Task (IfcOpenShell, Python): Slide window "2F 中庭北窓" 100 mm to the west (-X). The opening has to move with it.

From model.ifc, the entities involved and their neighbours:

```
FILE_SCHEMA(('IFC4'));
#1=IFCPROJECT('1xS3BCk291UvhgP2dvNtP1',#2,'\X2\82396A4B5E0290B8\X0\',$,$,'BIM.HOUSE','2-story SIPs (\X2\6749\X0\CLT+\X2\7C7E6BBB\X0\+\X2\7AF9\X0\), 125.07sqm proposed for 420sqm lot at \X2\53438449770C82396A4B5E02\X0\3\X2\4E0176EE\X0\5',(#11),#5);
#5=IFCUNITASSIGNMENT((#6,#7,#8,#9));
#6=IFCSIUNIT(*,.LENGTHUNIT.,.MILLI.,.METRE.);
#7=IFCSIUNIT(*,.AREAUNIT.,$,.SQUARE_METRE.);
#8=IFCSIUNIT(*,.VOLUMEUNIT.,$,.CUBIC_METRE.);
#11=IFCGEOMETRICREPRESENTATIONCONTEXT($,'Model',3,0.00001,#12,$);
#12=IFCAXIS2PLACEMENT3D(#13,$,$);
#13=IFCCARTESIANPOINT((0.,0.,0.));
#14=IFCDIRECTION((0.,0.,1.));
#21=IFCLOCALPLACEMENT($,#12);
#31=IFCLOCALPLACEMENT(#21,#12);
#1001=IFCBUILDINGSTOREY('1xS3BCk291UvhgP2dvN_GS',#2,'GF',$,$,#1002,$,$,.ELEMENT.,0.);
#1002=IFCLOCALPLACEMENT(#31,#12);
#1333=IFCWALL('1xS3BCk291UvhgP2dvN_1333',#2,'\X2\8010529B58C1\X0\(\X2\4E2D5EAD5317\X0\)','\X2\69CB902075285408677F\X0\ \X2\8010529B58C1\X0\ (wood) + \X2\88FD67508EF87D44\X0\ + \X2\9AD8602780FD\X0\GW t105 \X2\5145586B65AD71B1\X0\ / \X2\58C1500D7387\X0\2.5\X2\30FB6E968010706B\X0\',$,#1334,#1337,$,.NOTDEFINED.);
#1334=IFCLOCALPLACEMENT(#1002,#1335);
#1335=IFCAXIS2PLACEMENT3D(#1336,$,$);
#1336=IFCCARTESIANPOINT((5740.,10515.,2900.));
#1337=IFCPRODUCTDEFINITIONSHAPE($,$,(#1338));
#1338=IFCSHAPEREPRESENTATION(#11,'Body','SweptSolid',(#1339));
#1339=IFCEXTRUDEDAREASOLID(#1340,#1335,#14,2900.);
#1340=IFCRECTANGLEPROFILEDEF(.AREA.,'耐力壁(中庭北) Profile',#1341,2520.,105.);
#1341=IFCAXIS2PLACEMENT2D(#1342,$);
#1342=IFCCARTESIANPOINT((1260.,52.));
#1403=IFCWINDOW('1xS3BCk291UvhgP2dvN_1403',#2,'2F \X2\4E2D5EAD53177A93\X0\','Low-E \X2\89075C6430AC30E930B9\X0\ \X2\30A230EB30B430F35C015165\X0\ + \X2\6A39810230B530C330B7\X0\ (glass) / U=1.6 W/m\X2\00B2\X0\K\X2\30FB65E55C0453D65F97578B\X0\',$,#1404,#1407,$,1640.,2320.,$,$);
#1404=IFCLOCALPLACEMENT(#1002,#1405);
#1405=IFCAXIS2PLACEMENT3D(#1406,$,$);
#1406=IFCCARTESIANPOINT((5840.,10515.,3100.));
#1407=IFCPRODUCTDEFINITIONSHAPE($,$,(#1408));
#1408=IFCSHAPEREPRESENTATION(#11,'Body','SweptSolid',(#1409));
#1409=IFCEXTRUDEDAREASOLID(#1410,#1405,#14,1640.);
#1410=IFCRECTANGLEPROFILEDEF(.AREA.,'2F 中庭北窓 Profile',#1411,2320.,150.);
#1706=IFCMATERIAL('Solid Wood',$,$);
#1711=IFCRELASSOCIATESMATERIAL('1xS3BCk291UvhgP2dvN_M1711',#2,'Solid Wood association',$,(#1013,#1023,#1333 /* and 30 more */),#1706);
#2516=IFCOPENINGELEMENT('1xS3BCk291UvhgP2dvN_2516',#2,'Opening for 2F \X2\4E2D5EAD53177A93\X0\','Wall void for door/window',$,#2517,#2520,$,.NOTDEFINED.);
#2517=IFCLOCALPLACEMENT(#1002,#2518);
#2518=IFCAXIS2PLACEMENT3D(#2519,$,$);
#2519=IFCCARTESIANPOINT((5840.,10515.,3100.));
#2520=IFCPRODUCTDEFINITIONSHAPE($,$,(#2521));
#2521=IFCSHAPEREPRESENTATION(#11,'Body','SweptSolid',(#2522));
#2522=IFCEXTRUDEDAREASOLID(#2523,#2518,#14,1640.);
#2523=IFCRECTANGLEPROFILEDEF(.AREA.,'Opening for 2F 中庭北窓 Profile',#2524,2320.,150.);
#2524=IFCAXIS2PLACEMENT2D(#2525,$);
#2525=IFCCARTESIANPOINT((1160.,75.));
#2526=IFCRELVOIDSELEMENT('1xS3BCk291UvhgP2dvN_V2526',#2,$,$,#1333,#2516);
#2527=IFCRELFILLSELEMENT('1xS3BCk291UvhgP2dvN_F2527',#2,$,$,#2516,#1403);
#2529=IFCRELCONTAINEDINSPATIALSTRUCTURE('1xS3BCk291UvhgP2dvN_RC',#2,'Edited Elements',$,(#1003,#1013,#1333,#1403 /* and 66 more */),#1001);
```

```python
import ifcopenshell
import ifcopenshell.api.geometry
import ifcopenshell.util.placement
import ifcopenshell.util.unit

model = ifcopenshell.open("model.ifc")
unit_scale = ifcopenshell.util.unit.calculate_unit_scale(model)

window = model.by_guid("1xS3BCk291UvhgP2dvN_1403")
opening = window.FillsVoids[0].RelatingOpeningElement
wall = opening.VoidsElements[0].RelatingBuildingElement

wall_matrix = ifcopenshell.util.placement.get_local_placement(wall.ObjectPlacement)
shift = wall_matrix[:3, 0] * -0.1 / unit_scale
before = ifcopenshell.util.placement.get_local_placement(window.ObjectPlacement)[:3, 3].copy()

# The window is not placed relative to its opening, so move both.
for product in (opening, window):
    matrix = ifcopenshell.util.placement.get_local_placement(product.ObjectPlacement)
    matrix[:3, 3] += shift
    ifcopenshell.api.geometry.edit_object_placement(model, product=product, matrix=matrix, is_si=False)

after = ifcopenshell.util.placement.get_local_placement(window.ObjectPlacement)[:3, 3]
print("window moved by", (after - before).round(3) + 0.0)

model.write("model_edited.ifc")
```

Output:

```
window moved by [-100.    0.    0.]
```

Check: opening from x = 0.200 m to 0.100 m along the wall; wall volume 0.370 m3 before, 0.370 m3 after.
